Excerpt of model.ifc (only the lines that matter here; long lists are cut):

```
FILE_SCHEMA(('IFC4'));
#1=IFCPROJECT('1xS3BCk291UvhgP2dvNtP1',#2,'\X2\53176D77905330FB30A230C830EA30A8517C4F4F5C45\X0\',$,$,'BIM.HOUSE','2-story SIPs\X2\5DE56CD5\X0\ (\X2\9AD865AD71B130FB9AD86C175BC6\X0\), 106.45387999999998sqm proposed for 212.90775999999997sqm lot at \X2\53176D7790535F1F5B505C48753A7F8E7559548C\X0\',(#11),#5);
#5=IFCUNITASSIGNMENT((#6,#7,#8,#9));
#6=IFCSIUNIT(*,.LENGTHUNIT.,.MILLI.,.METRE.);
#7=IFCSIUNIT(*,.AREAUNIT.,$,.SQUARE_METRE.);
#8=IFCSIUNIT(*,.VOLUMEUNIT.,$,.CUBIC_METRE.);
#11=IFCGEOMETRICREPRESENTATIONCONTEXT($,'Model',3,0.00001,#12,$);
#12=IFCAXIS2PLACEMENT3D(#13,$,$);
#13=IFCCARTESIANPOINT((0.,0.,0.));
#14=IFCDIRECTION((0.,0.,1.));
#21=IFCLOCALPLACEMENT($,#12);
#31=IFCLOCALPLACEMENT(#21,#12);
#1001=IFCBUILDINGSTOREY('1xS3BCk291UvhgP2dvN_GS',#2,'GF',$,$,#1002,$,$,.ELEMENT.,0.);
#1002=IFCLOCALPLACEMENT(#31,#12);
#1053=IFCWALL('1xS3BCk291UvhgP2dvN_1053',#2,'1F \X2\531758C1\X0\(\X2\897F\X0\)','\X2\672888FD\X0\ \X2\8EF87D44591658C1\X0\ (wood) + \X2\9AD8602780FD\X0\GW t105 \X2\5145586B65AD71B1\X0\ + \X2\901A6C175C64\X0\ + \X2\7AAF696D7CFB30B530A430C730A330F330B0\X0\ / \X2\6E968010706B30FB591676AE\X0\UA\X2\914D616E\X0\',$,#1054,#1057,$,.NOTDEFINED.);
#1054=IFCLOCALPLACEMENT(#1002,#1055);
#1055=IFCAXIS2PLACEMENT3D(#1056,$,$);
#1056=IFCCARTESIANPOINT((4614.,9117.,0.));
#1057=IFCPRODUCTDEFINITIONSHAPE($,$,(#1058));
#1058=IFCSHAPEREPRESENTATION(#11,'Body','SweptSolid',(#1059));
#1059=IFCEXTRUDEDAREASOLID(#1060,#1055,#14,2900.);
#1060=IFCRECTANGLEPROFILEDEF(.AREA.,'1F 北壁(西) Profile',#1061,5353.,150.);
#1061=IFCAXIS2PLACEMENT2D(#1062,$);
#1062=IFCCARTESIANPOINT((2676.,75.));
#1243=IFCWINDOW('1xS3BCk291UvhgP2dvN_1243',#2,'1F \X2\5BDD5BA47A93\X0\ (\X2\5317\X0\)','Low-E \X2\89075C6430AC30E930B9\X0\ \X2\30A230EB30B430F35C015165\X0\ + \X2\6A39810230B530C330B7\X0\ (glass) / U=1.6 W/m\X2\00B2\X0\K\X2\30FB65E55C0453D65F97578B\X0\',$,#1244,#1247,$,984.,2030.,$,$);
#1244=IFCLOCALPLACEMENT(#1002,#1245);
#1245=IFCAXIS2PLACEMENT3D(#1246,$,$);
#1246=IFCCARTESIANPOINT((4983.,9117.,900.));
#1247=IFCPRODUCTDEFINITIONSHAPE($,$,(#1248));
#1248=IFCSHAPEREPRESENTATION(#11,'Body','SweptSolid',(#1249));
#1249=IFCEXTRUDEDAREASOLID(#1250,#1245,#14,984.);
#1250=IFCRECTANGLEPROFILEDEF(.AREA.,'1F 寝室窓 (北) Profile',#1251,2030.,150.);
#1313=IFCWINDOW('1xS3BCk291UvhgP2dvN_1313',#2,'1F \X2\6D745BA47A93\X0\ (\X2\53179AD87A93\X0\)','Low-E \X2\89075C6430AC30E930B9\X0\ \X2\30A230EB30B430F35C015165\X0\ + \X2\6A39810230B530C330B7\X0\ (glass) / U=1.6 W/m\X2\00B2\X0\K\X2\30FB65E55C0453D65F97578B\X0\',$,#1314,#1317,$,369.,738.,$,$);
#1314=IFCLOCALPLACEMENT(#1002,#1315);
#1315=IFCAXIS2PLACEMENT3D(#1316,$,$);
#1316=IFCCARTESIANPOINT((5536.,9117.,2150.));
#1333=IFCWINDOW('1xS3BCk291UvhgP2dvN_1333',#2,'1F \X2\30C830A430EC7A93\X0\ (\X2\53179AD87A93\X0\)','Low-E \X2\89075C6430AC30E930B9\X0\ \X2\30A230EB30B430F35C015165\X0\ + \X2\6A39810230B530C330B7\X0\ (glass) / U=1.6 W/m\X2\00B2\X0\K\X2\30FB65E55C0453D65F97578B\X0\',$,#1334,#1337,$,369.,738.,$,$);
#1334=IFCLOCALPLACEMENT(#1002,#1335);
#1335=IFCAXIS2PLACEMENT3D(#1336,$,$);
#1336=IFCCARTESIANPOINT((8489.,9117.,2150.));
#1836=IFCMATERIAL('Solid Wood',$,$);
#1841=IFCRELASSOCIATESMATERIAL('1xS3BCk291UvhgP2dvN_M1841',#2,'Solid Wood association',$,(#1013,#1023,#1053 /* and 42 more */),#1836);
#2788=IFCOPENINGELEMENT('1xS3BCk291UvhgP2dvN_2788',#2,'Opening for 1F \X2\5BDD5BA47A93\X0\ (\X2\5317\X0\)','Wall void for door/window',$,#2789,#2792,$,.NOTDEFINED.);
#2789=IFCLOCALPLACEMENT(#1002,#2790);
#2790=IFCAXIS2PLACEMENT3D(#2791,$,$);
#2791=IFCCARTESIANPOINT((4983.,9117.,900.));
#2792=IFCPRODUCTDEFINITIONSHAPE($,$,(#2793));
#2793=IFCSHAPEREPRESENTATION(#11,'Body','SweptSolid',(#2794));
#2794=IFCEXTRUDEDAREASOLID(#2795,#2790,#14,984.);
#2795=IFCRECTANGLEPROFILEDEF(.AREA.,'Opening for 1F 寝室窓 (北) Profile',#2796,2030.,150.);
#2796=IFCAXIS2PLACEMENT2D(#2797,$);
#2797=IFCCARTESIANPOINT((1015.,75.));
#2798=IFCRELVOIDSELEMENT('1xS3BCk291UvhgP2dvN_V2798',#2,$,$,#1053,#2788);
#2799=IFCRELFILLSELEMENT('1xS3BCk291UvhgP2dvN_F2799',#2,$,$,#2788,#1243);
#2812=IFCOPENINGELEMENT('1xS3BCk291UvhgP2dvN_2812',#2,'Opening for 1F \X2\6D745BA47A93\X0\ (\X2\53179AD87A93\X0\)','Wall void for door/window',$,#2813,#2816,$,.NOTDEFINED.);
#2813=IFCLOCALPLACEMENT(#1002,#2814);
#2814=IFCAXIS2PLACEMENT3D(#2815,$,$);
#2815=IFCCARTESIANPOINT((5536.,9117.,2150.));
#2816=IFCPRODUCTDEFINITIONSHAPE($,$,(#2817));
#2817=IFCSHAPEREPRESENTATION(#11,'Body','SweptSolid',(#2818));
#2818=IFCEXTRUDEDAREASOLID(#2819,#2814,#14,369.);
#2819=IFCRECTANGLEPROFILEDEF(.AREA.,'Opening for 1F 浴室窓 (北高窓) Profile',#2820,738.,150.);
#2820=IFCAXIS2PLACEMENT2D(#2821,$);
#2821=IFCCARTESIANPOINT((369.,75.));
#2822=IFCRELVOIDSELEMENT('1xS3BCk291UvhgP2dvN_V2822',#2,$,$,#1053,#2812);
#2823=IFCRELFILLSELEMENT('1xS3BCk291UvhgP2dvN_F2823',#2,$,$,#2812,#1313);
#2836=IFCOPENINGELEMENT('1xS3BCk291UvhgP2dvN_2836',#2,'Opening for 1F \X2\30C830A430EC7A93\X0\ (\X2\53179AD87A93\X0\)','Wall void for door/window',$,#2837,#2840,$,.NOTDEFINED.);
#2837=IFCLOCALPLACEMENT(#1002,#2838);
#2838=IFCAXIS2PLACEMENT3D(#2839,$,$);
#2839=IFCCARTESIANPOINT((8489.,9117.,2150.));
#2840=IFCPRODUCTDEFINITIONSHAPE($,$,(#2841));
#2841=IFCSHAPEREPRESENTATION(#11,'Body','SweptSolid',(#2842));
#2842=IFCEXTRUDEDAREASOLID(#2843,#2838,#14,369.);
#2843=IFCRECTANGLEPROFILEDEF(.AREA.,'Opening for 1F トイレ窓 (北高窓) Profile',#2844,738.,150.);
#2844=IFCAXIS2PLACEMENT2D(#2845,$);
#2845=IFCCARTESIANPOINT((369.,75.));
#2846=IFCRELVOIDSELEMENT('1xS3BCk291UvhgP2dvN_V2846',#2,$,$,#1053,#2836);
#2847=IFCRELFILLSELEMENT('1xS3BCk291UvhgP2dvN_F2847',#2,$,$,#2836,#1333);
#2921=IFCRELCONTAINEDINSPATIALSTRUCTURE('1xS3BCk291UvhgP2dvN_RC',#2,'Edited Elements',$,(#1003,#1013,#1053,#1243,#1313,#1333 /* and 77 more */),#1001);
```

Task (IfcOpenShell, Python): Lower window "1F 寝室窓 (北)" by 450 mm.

```python
import numpy as np
import ifcopenshell
import ifcopenshell.api.geometry
import ifcopenshell.util.placement
import ifcopenshell.util.unit

model = ifcopenshell.open("model.ifc")
unit_scale = ifcopenshell.util.unit.calculate_unit_scale(model)

window = model.by_id(1243)
opening = window.FillsVoids[0].RelatingOpeningElement
dz = -450.0

shift = np.array([0.0, 0.0, dz])
# The window is not placed relative to its opening, so move both.
for product in (opening, window):
    matrix = ifcopenshell.util.placement.get_local_placement(product.ObjectPlacement)
    matrix[:3, 3] += shift
    ifcopenshell.api.geometry.edit_object_placement(model, product=product, matrix=matrix, is_si=False)

print(f"moved by {dz * unit_scale:+.3f} m")

model.write("model_rev.ifc")
```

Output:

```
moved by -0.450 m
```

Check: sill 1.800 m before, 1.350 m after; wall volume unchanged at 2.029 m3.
